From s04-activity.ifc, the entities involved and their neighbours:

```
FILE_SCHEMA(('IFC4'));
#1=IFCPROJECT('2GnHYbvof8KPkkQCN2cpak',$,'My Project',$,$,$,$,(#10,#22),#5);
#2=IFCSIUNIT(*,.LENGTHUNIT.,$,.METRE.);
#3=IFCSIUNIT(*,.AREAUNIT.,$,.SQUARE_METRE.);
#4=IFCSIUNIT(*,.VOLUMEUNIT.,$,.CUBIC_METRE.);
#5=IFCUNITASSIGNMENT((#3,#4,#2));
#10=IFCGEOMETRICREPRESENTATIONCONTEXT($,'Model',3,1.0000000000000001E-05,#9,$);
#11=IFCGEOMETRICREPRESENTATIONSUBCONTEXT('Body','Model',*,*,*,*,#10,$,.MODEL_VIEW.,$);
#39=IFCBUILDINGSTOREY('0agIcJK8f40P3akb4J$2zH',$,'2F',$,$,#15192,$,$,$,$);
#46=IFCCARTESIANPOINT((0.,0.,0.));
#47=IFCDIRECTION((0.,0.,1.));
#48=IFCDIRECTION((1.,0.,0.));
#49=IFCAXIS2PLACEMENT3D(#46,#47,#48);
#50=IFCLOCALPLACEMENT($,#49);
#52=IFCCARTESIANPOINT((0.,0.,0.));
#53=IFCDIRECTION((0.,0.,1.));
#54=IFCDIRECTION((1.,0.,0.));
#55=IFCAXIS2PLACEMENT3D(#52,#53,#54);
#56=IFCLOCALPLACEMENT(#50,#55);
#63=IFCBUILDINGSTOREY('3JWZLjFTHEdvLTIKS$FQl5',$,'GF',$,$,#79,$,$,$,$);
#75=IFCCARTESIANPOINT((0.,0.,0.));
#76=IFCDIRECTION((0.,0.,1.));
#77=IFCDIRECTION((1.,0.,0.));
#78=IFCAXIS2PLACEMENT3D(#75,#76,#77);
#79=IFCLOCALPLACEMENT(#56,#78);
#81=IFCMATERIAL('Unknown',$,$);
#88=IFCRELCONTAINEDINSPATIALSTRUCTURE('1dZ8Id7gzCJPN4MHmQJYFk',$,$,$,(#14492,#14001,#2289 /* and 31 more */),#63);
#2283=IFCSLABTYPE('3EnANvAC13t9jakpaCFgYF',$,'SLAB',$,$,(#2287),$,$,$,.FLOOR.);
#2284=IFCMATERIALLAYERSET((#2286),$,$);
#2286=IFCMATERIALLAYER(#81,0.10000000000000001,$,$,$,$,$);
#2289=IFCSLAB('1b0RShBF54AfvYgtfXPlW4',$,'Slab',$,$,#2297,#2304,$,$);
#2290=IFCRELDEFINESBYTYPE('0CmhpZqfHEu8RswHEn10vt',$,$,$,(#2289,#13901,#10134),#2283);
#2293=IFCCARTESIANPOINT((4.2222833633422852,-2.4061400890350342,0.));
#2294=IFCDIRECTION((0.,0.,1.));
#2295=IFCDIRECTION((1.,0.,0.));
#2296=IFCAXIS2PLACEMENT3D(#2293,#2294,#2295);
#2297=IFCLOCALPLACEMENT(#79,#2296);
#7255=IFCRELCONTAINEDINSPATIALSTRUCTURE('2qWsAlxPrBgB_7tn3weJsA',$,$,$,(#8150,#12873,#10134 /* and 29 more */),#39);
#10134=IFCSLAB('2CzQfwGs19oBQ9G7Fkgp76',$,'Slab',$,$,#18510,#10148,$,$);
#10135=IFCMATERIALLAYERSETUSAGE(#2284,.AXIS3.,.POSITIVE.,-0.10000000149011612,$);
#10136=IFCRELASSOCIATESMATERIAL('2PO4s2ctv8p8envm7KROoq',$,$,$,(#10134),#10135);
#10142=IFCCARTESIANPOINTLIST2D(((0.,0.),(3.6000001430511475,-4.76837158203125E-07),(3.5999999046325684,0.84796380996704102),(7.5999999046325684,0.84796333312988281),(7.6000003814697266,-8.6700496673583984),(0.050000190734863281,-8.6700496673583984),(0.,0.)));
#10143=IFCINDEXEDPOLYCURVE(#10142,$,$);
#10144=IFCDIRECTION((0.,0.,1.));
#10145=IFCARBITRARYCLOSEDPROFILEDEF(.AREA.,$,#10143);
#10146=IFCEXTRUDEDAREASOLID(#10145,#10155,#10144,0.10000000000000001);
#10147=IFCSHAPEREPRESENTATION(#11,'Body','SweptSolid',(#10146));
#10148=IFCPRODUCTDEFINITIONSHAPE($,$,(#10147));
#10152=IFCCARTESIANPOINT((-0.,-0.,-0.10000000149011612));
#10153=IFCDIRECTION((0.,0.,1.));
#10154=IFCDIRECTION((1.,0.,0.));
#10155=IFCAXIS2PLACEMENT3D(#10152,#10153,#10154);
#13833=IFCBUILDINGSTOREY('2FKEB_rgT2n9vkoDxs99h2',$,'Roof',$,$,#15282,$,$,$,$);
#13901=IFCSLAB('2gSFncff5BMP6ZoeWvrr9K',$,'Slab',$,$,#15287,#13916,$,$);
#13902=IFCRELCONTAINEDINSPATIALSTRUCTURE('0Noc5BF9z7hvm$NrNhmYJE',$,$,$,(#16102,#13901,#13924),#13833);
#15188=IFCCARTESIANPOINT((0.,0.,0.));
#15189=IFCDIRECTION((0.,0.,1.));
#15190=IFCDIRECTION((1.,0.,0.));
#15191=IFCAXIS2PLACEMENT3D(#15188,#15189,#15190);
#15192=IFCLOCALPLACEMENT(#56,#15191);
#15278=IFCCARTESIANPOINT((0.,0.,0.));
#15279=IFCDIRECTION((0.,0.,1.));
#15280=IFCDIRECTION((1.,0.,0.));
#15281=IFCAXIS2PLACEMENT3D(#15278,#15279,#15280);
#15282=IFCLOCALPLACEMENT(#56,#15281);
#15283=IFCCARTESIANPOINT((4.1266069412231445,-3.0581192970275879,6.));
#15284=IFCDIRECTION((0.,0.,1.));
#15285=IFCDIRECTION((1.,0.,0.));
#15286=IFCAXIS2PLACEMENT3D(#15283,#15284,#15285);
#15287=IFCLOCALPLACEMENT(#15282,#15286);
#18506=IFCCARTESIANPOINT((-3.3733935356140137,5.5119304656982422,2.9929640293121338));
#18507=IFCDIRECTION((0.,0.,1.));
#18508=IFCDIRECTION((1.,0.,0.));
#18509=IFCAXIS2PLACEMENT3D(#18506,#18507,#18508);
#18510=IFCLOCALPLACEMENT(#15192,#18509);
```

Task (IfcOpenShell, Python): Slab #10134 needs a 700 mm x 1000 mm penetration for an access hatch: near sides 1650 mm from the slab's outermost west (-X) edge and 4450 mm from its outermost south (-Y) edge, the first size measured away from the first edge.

```python
import numpy as np
import ifcopenshell
import ifcopenshell.api.feature
import ifcopenshell.api.geometry
import ifcopenshell.api.root
import ifcopenshell.geom
import ifcopenshell.util.placement
import ifcopenshell.util.representation
import ifcopenshell.util.shape
import ifcopenshell.util.unit

model = ifcopenshell.open("s04-activity.ifc")
unit_scale = ifcopenshell.util.unit.calculate_unit_scale(model)
settings = ifcopenshell.geom.settings()


def volume(element):
    """Net volume in cubic metres, openings subtracted."""
    shape = ifcopenshell.geom.create_shape(settings, element)
    return ifcopenshell.util.shape.get_volume(shape.geometry)


slab = model.by_guid("2CzQfwGs19oBQ9G7Fkgp76")
before = volume(slab)

# Extent in the slab's own axes, in metres. The edges named are its -X and -Y sides.
slab_shape = ifcopenshell.geom.create_shape(settings, slab)
vertices = ifcopenshell.util.shape.get_vertices(slab_shape.geometry)
x_min, y_min, bottom = vertices.min(axis=0)
top = vertices[:, 2].max()

opening = ifcopenshell.api.root.create_entity(model, ifc_class="IfcOpeningElement", name="Access hatch opening", predefined_type="OPENING")
context = ifcopenshell.util.representation.get_context(model, "Model", "Body", "MODEL_VIEW")
width, depth = 0.7, 1
outline = [(0.0, 0.0), (width, 0.0), (width, depth), (0.0, depth), (0.0, 0.0)]
# Overshoot both faces by 50 mm so the cut is clean.
shape = ifcopenshell.api.geometry.add_slab_representation(
    model, context=context, depth=top - bottom + 0.1, polyline=outline
)
ifcopenshell.api.geometry.assign_representation(model, product=opening, representation=shape)

matrix = ifcopenshell.util.placement.get_local_placement(slab.ObjectPlacement)
matrix[:, 3] = matrix @ np.append(np.array([x_min + 1.65, y_min + 4.45, bottom - 0.05]) / unit_scale, 1.0)
ifcopenshell.api.geometry.edit_object_placement(model, product=opening, matrix=matrix, is_si=False)
ifcopenshell.api.feature.add_feature(model, feature=opening, element=slab)

after = volume(slab)

print(f"slab volume {before:.3f} -> {after:.3f} m3")

model.write("s04-activity_v2.ifc")
```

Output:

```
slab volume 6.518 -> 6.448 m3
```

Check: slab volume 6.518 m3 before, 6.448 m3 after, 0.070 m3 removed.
